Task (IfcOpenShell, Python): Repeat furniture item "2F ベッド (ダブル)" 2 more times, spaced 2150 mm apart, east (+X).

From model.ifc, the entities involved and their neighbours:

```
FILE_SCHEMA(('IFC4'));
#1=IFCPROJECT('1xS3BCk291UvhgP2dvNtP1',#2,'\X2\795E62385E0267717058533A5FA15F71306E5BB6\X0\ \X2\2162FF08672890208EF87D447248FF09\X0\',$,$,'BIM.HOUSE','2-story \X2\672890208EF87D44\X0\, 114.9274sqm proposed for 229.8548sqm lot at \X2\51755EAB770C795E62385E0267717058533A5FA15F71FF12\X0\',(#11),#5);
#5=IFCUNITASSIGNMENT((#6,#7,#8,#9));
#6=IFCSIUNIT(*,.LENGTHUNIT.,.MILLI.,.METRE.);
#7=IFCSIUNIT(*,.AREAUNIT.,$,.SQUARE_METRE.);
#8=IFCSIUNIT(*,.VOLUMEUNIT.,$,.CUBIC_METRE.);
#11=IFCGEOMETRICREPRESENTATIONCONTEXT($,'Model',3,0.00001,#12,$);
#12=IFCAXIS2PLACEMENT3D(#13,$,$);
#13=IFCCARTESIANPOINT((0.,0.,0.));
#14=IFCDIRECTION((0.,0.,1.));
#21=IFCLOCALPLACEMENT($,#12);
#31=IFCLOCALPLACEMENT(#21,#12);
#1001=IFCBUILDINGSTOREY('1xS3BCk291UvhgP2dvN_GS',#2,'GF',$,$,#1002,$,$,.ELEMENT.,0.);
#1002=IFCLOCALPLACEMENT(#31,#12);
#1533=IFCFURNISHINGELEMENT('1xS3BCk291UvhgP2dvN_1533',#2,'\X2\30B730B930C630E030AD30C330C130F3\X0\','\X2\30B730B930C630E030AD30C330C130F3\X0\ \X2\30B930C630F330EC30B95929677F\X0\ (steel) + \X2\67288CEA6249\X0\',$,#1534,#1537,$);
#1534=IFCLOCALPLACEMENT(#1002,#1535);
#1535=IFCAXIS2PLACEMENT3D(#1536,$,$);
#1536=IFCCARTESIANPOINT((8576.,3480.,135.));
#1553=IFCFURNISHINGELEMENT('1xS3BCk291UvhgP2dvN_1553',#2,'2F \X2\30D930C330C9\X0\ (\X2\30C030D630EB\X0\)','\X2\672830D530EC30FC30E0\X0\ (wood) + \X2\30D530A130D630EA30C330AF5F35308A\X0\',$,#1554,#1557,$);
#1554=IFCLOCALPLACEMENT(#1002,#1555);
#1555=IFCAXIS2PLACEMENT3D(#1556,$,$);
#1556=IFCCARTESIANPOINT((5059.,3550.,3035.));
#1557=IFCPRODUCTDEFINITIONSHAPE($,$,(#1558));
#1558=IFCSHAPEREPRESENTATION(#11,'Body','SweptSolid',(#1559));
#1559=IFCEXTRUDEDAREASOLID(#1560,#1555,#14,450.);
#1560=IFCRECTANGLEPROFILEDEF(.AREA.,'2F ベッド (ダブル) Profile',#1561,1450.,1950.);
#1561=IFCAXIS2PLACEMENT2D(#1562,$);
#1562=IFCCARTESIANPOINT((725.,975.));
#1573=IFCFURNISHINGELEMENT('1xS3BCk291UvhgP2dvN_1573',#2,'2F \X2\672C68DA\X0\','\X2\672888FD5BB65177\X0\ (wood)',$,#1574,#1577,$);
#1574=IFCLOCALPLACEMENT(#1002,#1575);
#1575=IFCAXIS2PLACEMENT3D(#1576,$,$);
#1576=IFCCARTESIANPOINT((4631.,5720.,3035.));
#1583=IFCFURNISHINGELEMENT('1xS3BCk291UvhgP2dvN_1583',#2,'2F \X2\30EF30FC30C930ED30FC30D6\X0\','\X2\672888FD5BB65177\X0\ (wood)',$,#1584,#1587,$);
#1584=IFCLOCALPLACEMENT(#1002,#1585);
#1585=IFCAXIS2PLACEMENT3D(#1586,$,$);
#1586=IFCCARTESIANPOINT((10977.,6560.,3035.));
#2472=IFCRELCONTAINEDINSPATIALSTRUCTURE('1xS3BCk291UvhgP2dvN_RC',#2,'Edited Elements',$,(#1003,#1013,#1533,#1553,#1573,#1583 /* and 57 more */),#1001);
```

```python
import numpy as np
import ifcopenshell
import ifcopenshell.api.geometry
import ifcopenshell.api.root
import ifcopenshell.util.element
import ifcopenshell.util.placement
import ifcopenshell.util.unit

model = ifcopenshell.open("model.ifc")
unit_scale = ifcopenshell.util.unit.calculate_unit_scale(model)


def reuse_history(source, copy):
    """copy_class also copies each property set's owner history, people and application; keep the originals."""
    for rel in copy.IsDefinedBy:
        if rel.is_a("IfcRelDefinesByProperties") and (history := rel.RelatingPropertyDefinition.OwnerHistory):
            rel.RelatingPropertyDefinition.OwnerHistory = source.OwnerHistory
            ifcopenshell.util.element.remove_deep2(model, history)


source = model.by_id(1553)
base = ifcopenshell.util.placement.get_local_placement(source.ObjectPlacement)
step = np.array([1.0, 0.0, 0.0]) * 2.15 / unit_scale

for i in range(1, 3):
    copy = ifcopenshell.api.root.copy_class(model, product=source)
    copy.Representation = ifcopenshell.util.element.copy_deep(
        model, source.Representation, exclude=["IfcGeometricRepresentationContext", "IfcRepresentationMap"]
    )
    reuse_history(source, copy)
    matrix = base.copy()
    matrix[:3, 3] += i * step
    print("added at", matrix[:3, 3].round(3) + 0.0)
    ifcopenshell.api.geometry.edit_object_placement(model, product=copy, matrix=matrix, is_si=False)

model.write("model_v2.ifc")
```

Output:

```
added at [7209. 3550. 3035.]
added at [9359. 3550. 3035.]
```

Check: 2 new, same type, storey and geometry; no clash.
